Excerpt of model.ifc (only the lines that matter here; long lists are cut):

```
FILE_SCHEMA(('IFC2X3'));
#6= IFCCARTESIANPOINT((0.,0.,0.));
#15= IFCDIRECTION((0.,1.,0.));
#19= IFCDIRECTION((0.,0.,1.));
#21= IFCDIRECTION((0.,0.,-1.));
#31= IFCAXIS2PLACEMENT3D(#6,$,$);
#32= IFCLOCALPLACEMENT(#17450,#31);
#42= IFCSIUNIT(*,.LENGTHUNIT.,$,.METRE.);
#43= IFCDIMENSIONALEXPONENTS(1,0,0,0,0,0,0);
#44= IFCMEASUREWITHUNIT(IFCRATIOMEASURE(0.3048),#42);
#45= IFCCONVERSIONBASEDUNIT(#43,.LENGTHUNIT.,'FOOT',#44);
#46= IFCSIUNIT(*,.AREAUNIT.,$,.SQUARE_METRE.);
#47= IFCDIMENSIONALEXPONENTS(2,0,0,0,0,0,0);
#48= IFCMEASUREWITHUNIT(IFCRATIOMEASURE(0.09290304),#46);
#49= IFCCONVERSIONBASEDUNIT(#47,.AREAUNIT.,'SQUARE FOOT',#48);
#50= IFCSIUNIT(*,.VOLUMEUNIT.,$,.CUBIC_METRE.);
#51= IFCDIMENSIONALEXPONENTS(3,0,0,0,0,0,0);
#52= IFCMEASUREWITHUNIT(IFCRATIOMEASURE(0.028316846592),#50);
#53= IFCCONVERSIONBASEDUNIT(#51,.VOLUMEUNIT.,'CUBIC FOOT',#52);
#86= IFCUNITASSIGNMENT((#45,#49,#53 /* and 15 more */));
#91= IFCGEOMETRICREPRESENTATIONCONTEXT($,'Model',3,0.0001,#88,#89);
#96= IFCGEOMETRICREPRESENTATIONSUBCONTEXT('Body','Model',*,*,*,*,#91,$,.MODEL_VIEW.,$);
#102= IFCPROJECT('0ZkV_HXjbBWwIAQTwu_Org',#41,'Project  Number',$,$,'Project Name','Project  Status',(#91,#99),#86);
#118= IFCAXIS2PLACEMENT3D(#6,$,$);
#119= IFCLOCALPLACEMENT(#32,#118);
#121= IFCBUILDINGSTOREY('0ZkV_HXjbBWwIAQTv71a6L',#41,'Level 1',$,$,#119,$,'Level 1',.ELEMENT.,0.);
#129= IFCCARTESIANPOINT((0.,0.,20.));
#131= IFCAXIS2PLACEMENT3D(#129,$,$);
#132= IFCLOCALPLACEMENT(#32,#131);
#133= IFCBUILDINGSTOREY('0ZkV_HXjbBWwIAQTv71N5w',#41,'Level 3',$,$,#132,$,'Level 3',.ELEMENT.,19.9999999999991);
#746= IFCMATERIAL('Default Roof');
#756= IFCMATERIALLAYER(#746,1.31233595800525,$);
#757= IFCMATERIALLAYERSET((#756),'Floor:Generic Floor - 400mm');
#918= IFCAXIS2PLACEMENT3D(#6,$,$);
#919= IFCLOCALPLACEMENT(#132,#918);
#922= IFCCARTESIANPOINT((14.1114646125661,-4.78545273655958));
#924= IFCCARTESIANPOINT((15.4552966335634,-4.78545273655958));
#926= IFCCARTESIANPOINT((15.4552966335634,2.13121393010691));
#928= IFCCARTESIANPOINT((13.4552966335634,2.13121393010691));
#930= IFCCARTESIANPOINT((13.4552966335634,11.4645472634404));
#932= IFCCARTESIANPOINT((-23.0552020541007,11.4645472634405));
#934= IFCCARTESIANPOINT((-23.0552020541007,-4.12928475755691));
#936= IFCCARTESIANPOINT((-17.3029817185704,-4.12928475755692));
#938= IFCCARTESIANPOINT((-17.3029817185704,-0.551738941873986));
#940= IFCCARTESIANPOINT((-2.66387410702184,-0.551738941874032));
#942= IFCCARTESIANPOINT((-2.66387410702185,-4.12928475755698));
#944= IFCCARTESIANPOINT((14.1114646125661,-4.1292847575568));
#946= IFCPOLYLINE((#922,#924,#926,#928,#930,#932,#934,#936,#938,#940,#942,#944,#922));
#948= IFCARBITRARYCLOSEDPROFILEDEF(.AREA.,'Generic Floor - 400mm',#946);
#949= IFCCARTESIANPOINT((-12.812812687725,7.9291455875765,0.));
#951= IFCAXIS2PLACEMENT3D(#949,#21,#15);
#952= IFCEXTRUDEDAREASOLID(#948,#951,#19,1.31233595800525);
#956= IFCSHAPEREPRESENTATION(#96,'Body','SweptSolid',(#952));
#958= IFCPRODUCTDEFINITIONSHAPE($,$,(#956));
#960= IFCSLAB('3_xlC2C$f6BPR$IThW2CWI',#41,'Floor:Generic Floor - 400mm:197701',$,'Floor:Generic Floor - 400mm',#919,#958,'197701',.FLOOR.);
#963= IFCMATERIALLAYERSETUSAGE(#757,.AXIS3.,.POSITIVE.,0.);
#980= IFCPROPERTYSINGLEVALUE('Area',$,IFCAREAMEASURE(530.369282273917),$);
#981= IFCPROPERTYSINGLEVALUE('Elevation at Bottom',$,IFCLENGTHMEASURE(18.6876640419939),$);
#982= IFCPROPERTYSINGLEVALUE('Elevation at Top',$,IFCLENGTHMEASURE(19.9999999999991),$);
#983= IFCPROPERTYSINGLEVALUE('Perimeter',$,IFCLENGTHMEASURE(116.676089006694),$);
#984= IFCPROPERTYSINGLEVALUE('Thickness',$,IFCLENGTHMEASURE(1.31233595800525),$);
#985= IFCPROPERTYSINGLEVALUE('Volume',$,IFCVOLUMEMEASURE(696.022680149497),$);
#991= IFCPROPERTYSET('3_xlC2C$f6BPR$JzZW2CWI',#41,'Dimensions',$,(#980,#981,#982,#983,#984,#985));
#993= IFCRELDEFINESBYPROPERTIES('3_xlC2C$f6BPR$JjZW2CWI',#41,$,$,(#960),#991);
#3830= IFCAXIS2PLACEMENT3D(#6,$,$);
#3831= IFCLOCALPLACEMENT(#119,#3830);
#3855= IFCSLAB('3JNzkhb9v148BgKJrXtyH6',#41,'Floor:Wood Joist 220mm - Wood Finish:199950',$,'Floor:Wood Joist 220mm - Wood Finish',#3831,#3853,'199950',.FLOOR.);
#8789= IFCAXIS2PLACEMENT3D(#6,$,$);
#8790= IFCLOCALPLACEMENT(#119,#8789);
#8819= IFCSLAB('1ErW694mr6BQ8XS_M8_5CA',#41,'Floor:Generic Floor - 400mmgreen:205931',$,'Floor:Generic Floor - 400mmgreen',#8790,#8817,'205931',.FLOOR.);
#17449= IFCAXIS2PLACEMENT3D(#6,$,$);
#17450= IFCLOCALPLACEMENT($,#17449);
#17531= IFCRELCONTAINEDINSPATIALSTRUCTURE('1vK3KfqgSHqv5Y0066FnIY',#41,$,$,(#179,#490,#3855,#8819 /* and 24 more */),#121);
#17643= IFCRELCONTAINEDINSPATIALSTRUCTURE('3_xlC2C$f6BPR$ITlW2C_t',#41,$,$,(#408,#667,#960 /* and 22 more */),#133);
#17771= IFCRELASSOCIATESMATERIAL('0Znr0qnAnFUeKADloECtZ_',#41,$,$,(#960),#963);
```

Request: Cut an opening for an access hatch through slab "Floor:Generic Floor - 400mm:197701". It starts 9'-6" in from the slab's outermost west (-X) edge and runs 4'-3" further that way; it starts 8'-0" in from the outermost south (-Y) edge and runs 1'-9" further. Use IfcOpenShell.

```python
import numpy as np
import ifcopenshell
import ifcopenshell.api.feature
import ifcopenshell.api.geometry
import ifcopenshell.api.pset
import ifcopenshell.api.root
import ifcopenshell.geom
import ifcopenshell.util.element
import ifcopenshell.util.placement
import ifcopenshell.util.representation
import ifcopenshell.util.shape
import ifcopenshell.util.unit

model = ifcopenshell.open("model.ifc")
unit_scale = ifcopenshell.util.unit.calculate_unit_scale(model)
area_scale = ifcopenshell.util.unit.calculate_unit_scale(model, "AREAUNIT")
volume_scale = ifcopenshell.util.unit.calculate_unit_scale(model, "VOLUMEUNIT")
settings = ifcopenshell.geom.settings()


def volume(element):
    """Net volume in cubic metres, openings subtracted."""
    shape = ifcopenshell.geom.create_shape(settings, element)
    return ifcopenshell.util.shape.get_volume(shape.geometry)


slab = model.by_guid("3_xlC2C$f6BPR$IThW2CWI")
before = volume(slab)

# Extent in the slab's own axes, in metres. The edges named are its -X and -Y sides.
slab_shape = ifcopenshell.geom.create_shape(settings, slab)
vertices = ifcopenshell.util.shape.get_vertices(slab_shape.geometry)
x_min, y_min, bottom = vertices.min(axis=0)
top = vertices[:, 2].max()

opening = ifcopenshell.api.root.create_entity(model, ifc_class="IfcOpeningElement", name="Access hatch opening")
context = ifcopenshell.util.representation.get_context(model, "Model", "Body", "MODEL_VIEW")
width, depth = 1.2954, 0.5334
outline = [(0.0, 0.0), (width, 0.0), (width, depth), (0.0, depth), (0.0, 0.0)]
# Overshoot both faces by 50 mm so the cut is clean.
shape = ifcopenshell.api.geometry.add_slab_representation(
    model, context=context, depth=top - bottom + 0.1, polyline=outline
)
ifcopenshell.api.geometry.assign_representation(model, product=opening, representation=shape)

matrix = ifcopenshell.util.placement.get_local_placement(slab.ObjectPlacement)
matrix[:, 3] = matrix @ np.append(np.array([x_min + 2.8956, y_min + 2.4384, bottom - 0.05]) / unit_scale, 1.0)
ifcopenshell.api.geometry.edit_object_placement(model, product=opening, matrix=matrix, is_si=False)
ifcopenshell.api.feature.add_feature(model, feature=opening, element=slab)

after = volume(slab)

# Update the slab's stored quantities.
pset = model.by_id(ifcopenshell.util.element.get_pset(slab, "Dimensions", should_inherit=False)["id"])
ifcopenshell.api.pset.edit_pset(model, pset=pset, properties={
    "Area": model.create_entity("IfcAreaMeasure", after / (top - bottom) / area_scale),
    "Volume": model.create_entity("IfcVolumeMeasure", after / volume_scale),
})

print(f"slab volume {before:.3f} -> {after:.3f} m3")

model.write("model_edited.ifc")
```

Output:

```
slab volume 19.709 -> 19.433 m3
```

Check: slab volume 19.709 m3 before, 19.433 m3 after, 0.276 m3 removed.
